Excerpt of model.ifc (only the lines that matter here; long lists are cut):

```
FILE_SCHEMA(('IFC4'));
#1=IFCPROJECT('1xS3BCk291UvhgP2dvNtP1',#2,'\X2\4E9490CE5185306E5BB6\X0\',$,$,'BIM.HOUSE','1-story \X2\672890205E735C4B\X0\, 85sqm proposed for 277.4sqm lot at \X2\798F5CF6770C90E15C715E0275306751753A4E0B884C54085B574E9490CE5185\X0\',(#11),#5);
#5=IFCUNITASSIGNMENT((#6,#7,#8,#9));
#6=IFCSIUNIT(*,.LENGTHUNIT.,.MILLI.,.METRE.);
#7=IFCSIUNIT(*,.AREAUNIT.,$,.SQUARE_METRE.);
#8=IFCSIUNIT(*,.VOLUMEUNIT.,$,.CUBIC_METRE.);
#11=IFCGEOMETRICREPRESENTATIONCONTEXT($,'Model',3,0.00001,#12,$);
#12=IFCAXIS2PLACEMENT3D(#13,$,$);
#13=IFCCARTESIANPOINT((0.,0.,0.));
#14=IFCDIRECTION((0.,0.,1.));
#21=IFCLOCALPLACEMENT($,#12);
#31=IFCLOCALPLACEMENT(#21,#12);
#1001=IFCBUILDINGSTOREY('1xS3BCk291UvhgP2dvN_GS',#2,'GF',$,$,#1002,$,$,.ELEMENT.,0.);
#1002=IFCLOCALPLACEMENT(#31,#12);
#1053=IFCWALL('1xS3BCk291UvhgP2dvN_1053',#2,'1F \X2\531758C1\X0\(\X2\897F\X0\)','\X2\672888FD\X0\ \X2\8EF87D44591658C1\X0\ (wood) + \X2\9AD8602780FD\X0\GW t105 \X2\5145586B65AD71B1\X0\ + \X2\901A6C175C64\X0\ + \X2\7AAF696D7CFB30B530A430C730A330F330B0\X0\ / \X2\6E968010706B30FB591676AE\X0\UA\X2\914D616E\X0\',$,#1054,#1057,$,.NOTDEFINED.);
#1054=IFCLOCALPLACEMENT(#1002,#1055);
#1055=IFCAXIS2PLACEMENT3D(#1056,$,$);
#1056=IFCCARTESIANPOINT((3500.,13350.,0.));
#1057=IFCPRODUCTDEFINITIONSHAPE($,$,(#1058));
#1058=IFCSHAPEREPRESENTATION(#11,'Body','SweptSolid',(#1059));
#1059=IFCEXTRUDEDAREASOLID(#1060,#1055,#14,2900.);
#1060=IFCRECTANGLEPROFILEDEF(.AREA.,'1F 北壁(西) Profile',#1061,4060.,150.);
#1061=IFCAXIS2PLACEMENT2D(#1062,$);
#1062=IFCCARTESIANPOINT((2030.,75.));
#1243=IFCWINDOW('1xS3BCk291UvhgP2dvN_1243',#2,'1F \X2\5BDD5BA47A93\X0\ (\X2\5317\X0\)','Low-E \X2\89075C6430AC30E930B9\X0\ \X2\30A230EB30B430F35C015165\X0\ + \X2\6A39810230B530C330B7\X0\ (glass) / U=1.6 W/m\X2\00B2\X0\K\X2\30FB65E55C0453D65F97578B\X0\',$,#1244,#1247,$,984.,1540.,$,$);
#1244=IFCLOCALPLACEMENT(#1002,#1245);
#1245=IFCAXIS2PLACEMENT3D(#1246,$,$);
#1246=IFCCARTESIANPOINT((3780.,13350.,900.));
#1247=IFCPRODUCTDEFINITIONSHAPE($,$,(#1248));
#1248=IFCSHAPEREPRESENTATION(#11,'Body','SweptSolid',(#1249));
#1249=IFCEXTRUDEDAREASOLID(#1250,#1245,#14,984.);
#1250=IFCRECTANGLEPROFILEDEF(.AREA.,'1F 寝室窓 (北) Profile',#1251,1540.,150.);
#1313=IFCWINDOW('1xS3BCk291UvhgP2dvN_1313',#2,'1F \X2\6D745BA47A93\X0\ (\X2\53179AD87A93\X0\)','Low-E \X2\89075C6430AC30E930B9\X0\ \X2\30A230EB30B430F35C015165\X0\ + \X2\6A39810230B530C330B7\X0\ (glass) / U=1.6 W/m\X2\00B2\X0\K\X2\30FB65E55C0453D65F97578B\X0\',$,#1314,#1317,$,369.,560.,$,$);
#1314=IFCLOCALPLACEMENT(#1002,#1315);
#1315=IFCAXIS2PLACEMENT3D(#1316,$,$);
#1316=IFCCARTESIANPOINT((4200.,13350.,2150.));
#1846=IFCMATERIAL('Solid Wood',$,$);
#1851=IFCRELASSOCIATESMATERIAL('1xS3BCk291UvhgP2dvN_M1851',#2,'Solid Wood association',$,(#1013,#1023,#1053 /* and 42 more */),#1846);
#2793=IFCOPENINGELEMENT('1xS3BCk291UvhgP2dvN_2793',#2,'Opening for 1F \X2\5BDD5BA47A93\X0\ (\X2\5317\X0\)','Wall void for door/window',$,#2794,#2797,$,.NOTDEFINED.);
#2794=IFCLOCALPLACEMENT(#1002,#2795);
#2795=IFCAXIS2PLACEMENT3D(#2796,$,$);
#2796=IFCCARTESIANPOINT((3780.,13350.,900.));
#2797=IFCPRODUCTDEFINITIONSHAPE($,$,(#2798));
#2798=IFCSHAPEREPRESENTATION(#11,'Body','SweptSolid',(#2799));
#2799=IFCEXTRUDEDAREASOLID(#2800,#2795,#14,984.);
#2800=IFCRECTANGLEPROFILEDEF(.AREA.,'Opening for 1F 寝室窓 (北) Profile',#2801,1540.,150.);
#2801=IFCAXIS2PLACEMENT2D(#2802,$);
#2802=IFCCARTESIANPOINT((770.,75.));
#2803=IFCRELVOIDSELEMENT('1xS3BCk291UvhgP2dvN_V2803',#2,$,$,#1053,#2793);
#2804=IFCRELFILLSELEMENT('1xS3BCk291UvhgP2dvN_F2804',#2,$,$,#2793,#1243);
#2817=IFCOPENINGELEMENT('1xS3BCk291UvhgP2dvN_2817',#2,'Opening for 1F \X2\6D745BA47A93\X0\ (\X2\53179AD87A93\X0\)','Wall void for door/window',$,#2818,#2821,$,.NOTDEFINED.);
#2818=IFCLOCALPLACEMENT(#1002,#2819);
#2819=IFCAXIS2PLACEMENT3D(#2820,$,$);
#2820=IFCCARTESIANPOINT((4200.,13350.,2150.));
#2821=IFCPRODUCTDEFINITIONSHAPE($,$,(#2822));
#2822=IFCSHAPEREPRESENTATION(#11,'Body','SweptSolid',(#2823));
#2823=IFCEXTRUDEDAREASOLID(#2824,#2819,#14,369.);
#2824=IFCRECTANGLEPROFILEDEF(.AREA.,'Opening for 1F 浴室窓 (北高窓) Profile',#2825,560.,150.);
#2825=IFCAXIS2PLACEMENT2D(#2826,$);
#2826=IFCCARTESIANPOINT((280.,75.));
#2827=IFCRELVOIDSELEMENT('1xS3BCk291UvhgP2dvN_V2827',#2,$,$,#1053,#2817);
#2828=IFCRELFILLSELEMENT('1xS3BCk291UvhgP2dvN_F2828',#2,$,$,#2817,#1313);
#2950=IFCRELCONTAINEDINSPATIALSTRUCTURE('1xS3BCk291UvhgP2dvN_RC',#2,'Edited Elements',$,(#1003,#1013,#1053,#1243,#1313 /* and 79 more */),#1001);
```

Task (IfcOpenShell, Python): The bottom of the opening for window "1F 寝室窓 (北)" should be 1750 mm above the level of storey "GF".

```python
import numpy as np
import ifcopenshell
import ifcopenshell.api.geometry
import ifcopenshell.geom
import ifcopenshell.util.element
import ifcopenshell.util.placement
import ifcopenshell.util.shape
import ifcopenshell.util.unit

model = ifcopenshell.open("model.ifc")
unit_scale = ifcopenshell.util.unit.calculate_unit_scale(model)

window = model.by_id(1243)
opening = window.FillsVoids[0].RelatingOpeningElement
storey = ifcopenshell.util.element.get_container(window, ifc_class="IfcBuildingStorey")
level = ifcopenshell.util.placement.get_local_placement(storey.ObjectPlacement)[2, 3]

# The opening's origin need not be at the sill, so measure its lowest point.
shape = ifcopenshell.geom.create_shape(ifcopenshell.geom.settings(), opening)
bottom = ifcopenshell.util.shape.get_shape_bottom_elevation(shape, shape.geometry) / unit_scale
dz = level + 1.75 / unit_scale - bottom

shift = np.array([0.0, 0.0, dz])
# The window is not placed relative to its opening, so move both.
for product in (opening, window):
    matrix = ifcopenshell.util.placement.get_local_placement(product.ObjectPlacement)
    matrix[:3, 3] += shift
    ifcopenshell.api.geometry.edit_object_placement(model, product=product, matrix=matrix, is_si=False)

print(f"moved by {dz * unit_scale:+.3f} m")

model.write("model_updated.ifc")
```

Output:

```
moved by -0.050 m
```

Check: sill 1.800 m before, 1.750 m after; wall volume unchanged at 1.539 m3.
